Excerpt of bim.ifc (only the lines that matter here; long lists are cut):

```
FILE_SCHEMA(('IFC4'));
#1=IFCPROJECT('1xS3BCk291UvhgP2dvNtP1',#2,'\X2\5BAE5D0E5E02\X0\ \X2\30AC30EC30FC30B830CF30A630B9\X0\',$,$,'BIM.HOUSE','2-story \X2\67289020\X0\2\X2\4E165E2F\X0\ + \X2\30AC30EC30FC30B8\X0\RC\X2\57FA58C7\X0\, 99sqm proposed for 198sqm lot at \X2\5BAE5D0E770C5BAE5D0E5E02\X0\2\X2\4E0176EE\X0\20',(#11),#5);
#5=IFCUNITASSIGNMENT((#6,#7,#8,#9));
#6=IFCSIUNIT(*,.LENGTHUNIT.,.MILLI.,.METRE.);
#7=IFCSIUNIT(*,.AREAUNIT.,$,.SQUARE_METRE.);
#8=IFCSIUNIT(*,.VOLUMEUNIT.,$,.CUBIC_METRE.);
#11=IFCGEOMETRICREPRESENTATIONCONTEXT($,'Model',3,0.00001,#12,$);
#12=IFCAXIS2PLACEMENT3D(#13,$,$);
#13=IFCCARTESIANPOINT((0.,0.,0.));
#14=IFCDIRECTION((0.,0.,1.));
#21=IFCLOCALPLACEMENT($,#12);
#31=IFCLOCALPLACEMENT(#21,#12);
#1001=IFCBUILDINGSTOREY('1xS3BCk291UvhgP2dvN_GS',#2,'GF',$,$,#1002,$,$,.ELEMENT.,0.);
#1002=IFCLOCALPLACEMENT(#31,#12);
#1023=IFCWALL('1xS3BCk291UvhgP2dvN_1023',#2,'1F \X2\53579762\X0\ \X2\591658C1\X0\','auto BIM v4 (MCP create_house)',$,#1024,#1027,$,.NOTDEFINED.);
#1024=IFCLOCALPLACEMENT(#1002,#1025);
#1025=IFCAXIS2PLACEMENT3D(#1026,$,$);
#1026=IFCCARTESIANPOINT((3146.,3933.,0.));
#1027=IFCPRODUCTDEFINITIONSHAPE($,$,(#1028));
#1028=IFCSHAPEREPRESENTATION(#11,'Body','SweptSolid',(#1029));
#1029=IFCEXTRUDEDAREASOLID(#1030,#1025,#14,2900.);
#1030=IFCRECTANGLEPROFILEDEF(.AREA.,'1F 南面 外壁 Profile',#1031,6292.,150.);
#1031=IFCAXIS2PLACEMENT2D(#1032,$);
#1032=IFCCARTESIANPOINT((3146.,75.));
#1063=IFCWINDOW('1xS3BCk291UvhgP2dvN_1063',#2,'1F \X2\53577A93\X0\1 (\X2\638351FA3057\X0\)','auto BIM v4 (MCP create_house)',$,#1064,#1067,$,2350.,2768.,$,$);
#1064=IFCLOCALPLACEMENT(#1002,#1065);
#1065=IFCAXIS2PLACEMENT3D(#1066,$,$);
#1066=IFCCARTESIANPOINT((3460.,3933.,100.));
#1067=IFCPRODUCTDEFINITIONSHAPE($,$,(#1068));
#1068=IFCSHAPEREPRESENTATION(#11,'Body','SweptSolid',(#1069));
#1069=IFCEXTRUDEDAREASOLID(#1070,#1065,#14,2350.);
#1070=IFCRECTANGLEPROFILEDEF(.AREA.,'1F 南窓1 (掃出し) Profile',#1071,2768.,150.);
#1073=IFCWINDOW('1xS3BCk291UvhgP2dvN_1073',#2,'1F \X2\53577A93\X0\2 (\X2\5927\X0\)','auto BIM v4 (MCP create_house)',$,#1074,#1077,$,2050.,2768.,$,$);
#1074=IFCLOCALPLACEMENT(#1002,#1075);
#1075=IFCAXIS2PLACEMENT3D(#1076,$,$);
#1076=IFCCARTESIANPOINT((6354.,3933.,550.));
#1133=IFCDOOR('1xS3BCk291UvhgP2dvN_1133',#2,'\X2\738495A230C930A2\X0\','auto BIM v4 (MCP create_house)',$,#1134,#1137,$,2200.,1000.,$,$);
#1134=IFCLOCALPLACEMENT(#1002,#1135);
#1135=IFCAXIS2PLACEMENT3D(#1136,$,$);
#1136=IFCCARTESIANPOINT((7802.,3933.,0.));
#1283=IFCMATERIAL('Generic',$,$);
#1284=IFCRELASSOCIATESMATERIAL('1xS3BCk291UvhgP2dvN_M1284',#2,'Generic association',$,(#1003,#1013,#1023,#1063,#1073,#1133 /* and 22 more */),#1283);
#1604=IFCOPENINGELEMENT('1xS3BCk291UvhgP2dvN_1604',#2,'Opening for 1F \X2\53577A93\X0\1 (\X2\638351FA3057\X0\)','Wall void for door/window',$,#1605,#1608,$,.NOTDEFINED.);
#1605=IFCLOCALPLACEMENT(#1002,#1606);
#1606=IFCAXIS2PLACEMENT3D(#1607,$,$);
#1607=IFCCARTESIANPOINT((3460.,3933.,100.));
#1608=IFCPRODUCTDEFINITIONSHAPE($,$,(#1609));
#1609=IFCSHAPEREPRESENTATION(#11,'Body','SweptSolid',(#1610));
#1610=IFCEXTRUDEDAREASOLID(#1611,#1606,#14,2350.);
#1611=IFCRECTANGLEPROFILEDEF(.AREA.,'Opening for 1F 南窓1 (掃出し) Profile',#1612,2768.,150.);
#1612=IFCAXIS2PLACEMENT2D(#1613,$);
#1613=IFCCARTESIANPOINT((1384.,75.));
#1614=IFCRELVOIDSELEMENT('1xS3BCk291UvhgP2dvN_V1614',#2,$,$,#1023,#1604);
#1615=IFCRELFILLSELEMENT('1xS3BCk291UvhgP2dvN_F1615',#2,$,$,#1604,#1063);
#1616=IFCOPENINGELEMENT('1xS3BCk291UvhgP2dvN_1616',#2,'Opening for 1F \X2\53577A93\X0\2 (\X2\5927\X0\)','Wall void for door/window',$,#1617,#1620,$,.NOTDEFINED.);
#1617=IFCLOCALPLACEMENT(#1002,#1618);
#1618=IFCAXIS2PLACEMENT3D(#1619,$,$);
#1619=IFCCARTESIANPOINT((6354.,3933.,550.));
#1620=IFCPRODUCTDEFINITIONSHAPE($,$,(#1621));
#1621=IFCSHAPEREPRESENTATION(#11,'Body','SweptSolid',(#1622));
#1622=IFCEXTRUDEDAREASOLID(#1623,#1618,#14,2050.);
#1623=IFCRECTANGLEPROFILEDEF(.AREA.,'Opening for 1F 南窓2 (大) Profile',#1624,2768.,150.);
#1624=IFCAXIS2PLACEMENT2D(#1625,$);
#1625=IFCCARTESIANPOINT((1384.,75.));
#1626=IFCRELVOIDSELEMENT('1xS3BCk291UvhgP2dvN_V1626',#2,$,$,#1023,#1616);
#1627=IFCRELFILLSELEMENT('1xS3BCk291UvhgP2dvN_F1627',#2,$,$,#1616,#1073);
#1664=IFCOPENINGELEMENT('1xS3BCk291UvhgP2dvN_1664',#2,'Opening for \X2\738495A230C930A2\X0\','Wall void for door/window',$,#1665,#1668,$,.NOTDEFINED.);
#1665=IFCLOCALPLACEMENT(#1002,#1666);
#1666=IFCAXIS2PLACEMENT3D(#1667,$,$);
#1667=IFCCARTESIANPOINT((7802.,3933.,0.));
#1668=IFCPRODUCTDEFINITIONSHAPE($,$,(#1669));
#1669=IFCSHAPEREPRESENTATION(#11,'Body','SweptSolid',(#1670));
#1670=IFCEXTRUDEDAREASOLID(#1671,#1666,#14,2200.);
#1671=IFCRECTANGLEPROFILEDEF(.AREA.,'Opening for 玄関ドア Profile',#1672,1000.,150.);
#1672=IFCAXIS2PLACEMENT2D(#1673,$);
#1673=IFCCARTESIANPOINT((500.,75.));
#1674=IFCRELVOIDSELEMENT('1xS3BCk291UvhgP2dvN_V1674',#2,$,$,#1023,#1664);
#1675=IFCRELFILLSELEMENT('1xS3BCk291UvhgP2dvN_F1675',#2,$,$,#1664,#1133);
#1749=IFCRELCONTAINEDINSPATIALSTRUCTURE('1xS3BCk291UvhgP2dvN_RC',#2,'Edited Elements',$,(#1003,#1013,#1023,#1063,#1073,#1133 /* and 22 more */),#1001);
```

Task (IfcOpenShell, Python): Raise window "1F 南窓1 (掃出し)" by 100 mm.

```python
import numpy as np
import ifcopenshell
import ifcopenshell.api.geometry
import ifcopenshell.util.placement
import ifcopenshell.util.unit

model = ifcopenshell.open("bim.ifc")
unit_scale = ifcopenshell.util.unit.calculate_unit_scale(model)

window = model.by_guid("1xS3BCk291UvhgP2dvN_1063")
opening = window.FillsVoids[0].RelatingOpeningElement
dz = 100.0

shift = np.array([0.0, 0.0, dz])
# The window is not placed relative to its opening, so move both.
for product in (opening, window):
    matrix = ifcopenshell.util.placement.get_local_placement(product.ObjectPlacement)
    matrix[:3, 3] += shift
    ifcopenshell.api.geometry.edit_object_placement(model, product=product, matrix=matrix, is_si=False)

print(f"moved by {dz * unit_scale:+.3f} m")

model.write("bim_edited.ifc")
```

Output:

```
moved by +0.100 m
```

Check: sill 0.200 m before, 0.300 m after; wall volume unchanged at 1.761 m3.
